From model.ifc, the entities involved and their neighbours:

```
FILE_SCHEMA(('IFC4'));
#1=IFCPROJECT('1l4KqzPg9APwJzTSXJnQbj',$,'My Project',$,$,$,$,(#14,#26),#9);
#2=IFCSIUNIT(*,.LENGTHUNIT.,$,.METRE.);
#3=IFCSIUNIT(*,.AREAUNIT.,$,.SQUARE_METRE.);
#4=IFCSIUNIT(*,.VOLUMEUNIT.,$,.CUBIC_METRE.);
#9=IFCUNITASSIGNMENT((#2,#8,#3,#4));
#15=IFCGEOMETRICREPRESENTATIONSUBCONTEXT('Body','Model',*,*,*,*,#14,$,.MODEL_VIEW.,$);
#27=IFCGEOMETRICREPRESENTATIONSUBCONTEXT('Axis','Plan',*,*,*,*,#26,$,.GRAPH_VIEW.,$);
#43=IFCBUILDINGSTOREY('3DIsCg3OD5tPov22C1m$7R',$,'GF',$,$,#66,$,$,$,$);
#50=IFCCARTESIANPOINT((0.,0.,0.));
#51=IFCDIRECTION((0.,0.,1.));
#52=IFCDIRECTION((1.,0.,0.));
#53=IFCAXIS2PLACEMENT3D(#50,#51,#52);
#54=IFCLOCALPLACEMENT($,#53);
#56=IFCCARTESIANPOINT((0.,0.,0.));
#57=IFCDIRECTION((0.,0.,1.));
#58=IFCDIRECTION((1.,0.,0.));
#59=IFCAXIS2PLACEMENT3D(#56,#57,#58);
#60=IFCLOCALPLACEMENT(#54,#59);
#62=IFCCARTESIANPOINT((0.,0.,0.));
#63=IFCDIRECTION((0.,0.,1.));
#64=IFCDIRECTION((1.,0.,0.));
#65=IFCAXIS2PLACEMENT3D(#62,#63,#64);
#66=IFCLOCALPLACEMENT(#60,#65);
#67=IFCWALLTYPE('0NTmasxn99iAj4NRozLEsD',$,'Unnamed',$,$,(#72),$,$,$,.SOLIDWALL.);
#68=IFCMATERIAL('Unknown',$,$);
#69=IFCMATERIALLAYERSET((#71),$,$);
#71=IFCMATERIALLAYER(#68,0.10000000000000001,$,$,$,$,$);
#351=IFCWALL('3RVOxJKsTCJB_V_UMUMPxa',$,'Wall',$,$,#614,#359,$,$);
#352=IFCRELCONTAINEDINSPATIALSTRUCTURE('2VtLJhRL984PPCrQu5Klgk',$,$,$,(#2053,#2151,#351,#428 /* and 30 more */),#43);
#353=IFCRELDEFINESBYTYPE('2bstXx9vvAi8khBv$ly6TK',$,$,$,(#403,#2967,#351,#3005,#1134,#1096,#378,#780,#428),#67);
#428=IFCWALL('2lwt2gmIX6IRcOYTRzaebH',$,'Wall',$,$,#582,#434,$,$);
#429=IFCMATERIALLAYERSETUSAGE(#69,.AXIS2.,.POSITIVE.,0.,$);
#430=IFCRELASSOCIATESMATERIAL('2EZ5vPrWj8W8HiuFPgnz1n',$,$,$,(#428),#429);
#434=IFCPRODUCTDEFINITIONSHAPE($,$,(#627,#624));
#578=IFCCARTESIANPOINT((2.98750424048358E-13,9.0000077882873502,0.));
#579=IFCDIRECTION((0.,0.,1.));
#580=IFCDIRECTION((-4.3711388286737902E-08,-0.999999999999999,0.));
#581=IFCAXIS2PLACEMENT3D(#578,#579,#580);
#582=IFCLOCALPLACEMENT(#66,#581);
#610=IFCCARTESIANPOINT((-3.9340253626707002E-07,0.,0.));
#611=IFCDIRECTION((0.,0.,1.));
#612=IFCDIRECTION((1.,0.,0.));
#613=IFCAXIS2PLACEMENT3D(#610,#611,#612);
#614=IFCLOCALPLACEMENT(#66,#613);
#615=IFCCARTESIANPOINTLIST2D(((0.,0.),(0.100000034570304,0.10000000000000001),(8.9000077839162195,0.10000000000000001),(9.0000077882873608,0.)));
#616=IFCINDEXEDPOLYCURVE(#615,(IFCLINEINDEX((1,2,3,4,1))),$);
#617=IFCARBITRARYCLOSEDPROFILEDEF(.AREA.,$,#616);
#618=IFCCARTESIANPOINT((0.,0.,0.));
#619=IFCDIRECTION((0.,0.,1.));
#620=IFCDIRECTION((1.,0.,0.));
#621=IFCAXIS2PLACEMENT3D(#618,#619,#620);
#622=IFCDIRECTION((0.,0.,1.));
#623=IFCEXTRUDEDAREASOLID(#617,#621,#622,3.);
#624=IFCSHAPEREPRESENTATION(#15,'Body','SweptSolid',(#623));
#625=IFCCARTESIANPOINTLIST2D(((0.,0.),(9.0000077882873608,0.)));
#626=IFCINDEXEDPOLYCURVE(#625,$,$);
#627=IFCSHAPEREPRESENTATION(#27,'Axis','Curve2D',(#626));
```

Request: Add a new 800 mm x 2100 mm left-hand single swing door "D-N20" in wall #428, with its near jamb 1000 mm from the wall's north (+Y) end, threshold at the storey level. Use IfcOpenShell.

```python
import numpy as np
import ifcopenshell
import ifcopenshell.api.feature
import ifcopenshell.api.geometry
import ifcopenshell.api.root
import ifcopenshell.api.spatial
import ifcopenshell.geom
import ifcopenshell.util.element
import ifcopenshell.util.placement
import ifcopenshell.util.representation
import ifcopenshell.util.shape
import ifcopenshell.util.unit

model = ifcopenshell.open("model.ifc")
unit_scale = ifcopenshell.util.unit.calculate_unit_scale(model)
settings = ifcopenshell.geom.settings()


def volume(element):
    """Net volume in cubic metres, openings subtracted."""
    shape = ifcopenshell.geom.create_shape(settings, element)
    return ifcopenshell.util.shape.get_volume(shape.geometry)


wall = model.by_guid("2lwt2gmIX6IRcOYTRzaebH")
storey = ifcopenshell.util.element.get_container(wall, ifc_class="IfcBuildingStorey")
context = ifcopenshell.util.representation.get_context(model, "Model", "Body", "MODEL_VIEW")
before = volume(wall)

width, height, from_end, sill = 0.8, 2.1, 1, 0.0  # metres

# The wall runs along its own X axis, and the end named is its -X end.
wall_shape = ifcopenshell.geom.create_shape(settings, wall)
x, y, z = ifcopenshell.util.shape.get_vertices(wall_shape.geometry).T
start = x.min() + from_end
face, thickness = float(y.min()), float(y.max() - y.min())
wall_matrix = ifcopenshell.util.placement.get_local_placement(wall.ObjectPlacement)
level = ifcopenshell.util.placement.get_local_placement(storey.ObjectPlacement)[2, 3]


def in_wall(x, y):
    """Placement at x, y metres in the wall's axes, at sill height."""
    matrix = wall_matrix.copy()
    matrix[:, 3] = wall_matrix @ np.array([x / unit_scale, y / unit_scale, 0.0, 1.0])
    matrix[2, 3] = level + sill / unit_scale
    return matrix


# Opening: a box that overshoots both wall faces by 50 mm.
opening = ifcopenshell.api.root.create_entity(model, ifc_class="IfcOpeningElement", predefined_type="OPENING")
box = ifcopenshell.api.geometry.add_wall_representation(
    model, context=context, length=width, height=height, thickness=thickness + 0.1
)
ifcopenshell.api.geometry.assign_representation(model, product=opening, representation=box)
ifcopenshell.api.geometry.edit_object_placement(model, product=opening, matrix=in_wall(start, face - 0.05), is_si=False)
ifcopenshell.api.feature.add_feature(model, feature=opening, element=wall)

door = ifcopenshell.api.root.create_entity(model, ifc_class="IfcDoor", name="D-N20", predefined_type="DOOR")
door.OverallWidth, door.OverallHeight = width / unit_scale, height / unit_scale
door.OperationType = "SINGLE_SWING_LEFT"
body = ifcopenshell.api.geometry.add_door_representation(
    model,
    context=context,
    overall_width=door.OverallWidth,
    overall_height=door.OverallHeight,
    operation_type="SINGLE_SWING_LEFT",
    lining_properties={"LiningDepth": thickness / unit_scale, "ThresholdDepth": thickness / unit_scale},
)
ifcopenshell.api.geometry.assign_representation(model, product=door, representation=body)
ifcopenshell.api.spatial.assign_container(model, products=[door], relating_structure=storey)
ifcopenshell.api.feature.add_filling(model, opening=opening, element=door)

# The lining spans the wall, so the door starts at the wall face.
ifcopenshell.api.geometry.edit_object_placement(model, product=door, matrix=in_wall(start, face), is_si=False)

after = volume(wall)

print(f"wall volume {before:.3f} -> {after:.3f} m3")

model.write("model_edited.ifc")
```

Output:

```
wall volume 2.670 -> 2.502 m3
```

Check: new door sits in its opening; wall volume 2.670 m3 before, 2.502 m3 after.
